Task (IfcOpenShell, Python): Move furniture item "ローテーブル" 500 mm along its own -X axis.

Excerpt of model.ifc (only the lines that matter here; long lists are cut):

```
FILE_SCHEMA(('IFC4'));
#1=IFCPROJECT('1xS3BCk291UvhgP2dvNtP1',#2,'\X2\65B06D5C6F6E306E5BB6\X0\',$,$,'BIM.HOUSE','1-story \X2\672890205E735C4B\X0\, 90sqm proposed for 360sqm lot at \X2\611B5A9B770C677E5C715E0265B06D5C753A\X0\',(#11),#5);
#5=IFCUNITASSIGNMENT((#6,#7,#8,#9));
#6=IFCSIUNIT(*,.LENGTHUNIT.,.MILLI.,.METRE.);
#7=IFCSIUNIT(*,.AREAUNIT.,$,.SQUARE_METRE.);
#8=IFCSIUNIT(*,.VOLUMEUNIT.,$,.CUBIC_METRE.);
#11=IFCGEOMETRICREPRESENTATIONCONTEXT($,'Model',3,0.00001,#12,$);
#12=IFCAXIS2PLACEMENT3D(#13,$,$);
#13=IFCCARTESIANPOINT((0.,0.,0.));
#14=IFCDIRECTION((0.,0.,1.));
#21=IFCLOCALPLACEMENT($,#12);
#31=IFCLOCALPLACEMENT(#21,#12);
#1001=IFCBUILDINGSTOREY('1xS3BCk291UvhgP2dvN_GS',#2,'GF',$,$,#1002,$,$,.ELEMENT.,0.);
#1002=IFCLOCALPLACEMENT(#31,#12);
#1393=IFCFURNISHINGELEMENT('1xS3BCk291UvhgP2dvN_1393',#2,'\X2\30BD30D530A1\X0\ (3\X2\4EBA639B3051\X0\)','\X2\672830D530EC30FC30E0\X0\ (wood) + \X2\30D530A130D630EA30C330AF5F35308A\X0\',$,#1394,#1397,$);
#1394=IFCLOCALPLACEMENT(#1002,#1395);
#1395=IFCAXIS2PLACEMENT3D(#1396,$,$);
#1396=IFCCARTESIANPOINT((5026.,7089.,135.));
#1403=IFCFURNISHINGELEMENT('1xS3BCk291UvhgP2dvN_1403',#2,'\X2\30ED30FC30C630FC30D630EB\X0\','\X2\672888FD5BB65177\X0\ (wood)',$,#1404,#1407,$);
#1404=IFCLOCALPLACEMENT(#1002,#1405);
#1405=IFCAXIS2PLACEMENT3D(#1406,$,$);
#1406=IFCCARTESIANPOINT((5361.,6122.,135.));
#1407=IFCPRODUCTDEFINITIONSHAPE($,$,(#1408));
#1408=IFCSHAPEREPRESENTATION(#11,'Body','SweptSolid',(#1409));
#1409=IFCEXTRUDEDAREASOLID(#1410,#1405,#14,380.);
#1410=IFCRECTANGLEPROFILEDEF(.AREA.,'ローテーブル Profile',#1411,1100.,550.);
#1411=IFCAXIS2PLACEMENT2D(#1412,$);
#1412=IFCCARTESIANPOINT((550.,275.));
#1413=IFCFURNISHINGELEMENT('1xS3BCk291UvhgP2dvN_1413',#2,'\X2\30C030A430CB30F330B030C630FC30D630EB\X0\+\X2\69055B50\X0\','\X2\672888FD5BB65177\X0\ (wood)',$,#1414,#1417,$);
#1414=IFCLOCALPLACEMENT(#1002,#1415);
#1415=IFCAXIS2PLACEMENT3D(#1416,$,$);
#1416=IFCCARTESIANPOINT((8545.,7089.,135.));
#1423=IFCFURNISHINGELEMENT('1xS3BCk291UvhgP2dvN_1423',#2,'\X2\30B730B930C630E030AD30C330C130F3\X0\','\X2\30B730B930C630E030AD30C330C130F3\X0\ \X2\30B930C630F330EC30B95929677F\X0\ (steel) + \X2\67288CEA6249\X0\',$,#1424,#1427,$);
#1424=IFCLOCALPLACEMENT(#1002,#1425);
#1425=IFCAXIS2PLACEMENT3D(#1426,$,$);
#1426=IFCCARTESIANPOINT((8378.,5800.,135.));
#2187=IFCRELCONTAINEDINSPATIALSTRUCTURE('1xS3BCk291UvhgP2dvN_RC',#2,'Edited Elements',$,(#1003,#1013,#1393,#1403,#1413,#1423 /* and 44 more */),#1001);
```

```python
import ifcopenshell
import ifcopenshell.api.geometry
import ifcopenshell.util.placement

model = ifcopenshell.open("model.ifc")

item = model.by_id(1403)
matrix = ifcopenshell.util.placement.get_local_placement(item.ObjectPlacement)
matrix[:3, 3] -= matrix[:3, 0] * 500.0
ifcopenshell.api.geometry.edit_object_placement(model, product=item, matrix=matrix, is_si=False)

print(ifcopenshell.util.placement.get_local_placement(item.ObjectPlacement).round(3) + 0.0)

model.write("model_rev.ifc")
```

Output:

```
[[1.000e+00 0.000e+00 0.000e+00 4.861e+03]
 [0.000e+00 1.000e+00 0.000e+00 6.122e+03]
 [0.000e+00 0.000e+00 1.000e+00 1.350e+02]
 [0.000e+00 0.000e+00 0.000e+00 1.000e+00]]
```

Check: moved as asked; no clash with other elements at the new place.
